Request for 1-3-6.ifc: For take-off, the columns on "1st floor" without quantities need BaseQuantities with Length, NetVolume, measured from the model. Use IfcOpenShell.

First a look at what the model holds.

```python
import ifcopenshell
import ifcopenshell.util.element
import ifcopenshell.util.unit

model = ifcopenshell.open("1-3-6.ifc")
print(model.schema)
for unit_type in ("LENGTHUNIT", "AREAUNIT", "VOLUMEUNIT"):
    print(unit_type, ifcopenshell.util.unit.calculate_unit_scale(model, unit_type))
storey = next(s for s in model.by_type("IfcBuildingStorey") if s.Name == "1st floor")
columns = [e for e in ifcopenshell.util.element.get_decomposition(storey) if e.is_a("IfcColumn")]
for e in sorted(columns, key=lambda e: e.id()):
    print(e.id(), e.is_a(), e.Name, list(ifcopenshell.util.element.get_psets(e, qtos_only=True)), sep=" | ")
```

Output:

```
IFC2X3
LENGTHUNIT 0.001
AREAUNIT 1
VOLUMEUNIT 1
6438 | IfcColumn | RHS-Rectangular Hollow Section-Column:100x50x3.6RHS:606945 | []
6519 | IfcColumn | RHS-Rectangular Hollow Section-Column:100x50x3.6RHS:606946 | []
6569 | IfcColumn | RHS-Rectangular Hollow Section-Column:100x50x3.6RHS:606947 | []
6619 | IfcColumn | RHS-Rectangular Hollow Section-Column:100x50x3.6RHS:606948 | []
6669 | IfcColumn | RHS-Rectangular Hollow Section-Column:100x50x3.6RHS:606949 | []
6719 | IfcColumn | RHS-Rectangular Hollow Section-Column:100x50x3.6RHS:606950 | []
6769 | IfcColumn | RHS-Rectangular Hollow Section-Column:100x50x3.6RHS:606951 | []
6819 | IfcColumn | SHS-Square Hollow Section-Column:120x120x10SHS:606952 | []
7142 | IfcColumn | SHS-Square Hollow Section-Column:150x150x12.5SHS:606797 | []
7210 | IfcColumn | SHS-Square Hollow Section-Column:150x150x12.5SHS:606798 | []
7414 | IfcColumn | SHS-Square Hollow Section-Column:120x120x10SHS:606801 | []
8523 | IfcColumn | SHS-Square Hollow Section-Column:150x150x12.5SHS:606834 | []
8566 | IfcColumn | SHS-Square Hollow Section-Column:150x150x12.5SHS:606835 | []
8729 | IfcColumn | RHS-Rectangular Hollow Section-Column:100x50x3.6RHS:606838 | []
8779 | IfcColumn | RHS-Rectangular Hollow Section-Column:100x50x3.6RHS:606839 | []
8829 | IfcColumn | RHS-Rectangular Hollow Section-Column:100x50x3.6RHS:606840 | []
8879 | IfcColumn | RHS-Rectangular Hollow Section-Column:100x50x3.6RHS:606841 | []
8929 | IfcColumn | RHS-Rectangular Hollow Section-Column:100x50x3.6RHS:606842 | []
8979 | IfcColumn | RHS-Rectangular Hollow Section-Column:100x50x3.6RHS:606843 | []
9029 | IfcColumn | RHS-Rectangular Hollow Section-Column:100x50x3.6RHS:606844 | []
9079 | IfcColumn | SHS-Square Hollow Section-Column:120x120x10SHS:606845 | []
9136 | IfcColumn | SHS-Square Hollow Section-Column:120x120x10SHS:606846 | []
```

```python
import ifcopenshell
import ifcopenshell.api.pset
import ifcopenshell.geom
import ifcopenshell.util.element
import ifcopenshell.util.shape
import ifcopenshell.util.unit

model = ifcopenshell.open("1-3-6.ifc")
unit_scale = ifcopenshell.util.unit.calculate_unit_scale(model)
volume_scale = ifcopenshell.util.unit.calculate_unit_scale(model, "VOLUMEUNIT")
settings = ifcopenshell.geom.settings()

storey = next(s for s in model.by_type("IfcBuildingStorey") if s.Name == "1st floor")
columns = [e for e in ifcopenshell.util.element.get_decomposition(storey) if e.is_a("IfcColumn")]

for e in sorted(columns, key=lambda e: e.id()):
    if ifcopenshell.util.element.get_psets(e, qtos_only=True, should_inherit=False):
        continue
    # Geometry comes back in metres, in the element's own axes.
    shape = ifcopenshell.geom.create_shape(settings, e)
    values = {
        "Length": ifcopenshell.util.shape.get_z(shape.geometry) / unit_scale,
        "NetVolume": ifcopenshell.util.shape.get_volume(shape.geometry) / volume_scale,
    }
    qto = ifcopenshell.api.pset.add_qto(model, product=e, name="BaseQuantities")
    ifcopenshell.api.pset.edit_qto(model, qto=qto, properties=values)
    print(e.id(), {k: round(v, 3) for k, v in values.items()})

model.write("1-3-6_v2.ifc")
```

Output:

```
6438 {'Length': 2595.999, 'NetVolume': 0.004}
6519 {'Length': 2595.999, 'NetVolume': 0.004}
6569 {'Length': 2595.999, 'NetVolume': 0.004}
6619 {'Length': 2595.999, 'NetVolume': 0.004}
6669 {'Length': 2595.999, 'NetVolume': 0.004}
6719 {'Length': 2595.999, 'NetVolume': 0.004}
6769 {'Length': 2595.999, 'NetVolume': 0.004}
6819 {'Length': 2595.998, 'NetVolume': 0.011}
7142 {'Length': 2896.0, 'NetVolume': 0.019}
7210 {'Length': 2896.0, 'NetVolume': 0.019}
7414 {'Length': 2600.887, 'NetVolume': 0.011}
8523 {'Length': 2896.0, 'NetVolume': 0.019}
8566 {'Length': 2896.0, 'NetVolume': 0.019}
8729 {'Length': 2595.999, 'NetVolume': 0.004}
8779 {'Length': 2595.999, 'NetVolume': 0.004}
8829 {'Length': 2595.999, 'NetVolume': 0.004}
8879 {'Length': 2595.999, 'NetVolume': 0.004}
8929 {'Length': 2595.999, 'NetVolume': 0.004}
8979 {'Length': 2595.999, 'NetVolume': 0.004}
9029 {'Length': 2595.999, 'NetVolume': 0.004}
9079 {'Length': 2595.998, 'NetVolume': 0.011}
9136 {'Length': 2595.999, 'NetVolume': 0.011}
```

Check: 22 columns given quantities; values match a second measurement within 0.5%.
